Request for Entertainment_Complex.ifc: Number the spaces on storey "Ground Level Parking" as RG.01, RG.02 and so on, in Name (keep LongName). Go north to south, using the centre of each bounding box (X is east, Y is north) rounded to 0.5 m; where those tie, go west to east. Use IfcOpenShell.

First a look at what the model holds.

```python
import ifcopenshell
import ifcopenshell.util.element
import ifcopenshell.util.placement

model = ifcopenshell.open("Entertainment_Complex.ifc")
print(model.schema)
storey = next(s for s in model.by_type("IfcBuildingStorey") if s.Name == "Ground Level Parking")
spaces = [e for e in ifcopenshell.util.element.get_decomposition(storey) if e.is_a("IfcSpace")]
for e in sorted(spaces, key=lambda e: e.id()):
    origin = ifcopenshell.util.placement.get_local_placement(e.ObjectPlacement)[:3, 3]
    print(e.id(), e.Name, e.LongName, origin.round(2) + 0.0, sep=" | ")
```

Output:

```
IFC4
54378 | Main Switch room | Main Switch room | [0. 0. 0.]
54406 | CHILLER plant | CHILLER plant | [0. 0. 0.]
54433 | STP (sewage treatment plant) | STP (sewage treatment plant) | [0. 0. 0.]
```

```python
import ifcopenshell
import ifcopenshell.geom
import ifcopenshell.util.element
import ifcopenshell.util.shape

model = ifcopenshell.open("Entertainment_Complex.ifc")
settings = ifcopenshell.geom.settings()
settings.set("use-world-coords", True)


def centre(element):
    shape = ifcopenshell.geom.create_shape(settings, element)
    return ifcopenshell.util.shape.get_bbox_centroid(shape.geometry)


storey = next(s for s in model.by_type("IfcBuildingStorey") if s.Name == "Ground Level Parking")
spaces = [e for e in ifcopenshell.util.element.get_decomposition(storey) if e.is_a("IfcSpace")]

# Insertion points can sit at a corner or the storey origin, so sort by the geometry (in metres).
centres = {e: centre(e) for e in spaces}
spaces.sort(key=lambda e: (-round(centres[e][1] / 0.5), centres[e][0]))

for i, e in enumerate(spaces, start=1):
    number = f"RG.{i:02d}"
    e.Name = number
    print(e.id(), number)

model.write("Entertainment_Complex_rev.ifc")
```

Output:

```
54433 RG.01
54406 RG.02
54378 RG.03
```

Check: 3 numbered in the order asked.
